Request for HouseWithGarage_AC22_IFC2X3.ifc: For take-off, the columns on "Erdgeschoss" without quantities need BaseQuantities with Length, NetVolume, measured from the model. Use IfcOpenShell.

First a look at what the model holds.

```python
import ifcopenshell
import ifcopenshell.util.element
import ifcopenshell.util.unit

model = ifcopenshell.open("HouseWithGarage_AC22_IFC2X3.ifc")
print(model.schema)
for unit_type in ("LENGTHUNIT", "AREAUNIT", "VOLUMEUNIT"):
    print(unit_type, ifcopenshell.util.unit.calculate_unit_scale(model, unit_type))
storey = next(s for s in model.by_type("IfcBuildingStorey") if s.Name == "Erdgeschoss")
columns = [e for e in ifcopenshell.util.element.get_decomposition(storey) if e.is_a("IfcColumn")]
for e in sorted(columns, key=lambda e: e.id()):
    print(e.id(), e.is_a(), e.Name, list(ifcopenshell.util.element.get_psets(e, qtos_only=True)), sep=" | ")
```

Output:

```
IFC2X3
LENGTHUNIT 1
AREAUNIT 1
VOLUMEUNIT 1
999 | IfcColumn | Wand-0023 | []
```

```python
import ifcopenshell
import ifcopenshell.api.pset
import ifcopenshell.geom
import ifcopenshell.util.element
import ifcopenshell.util.shape
import ifcopenshell.util.unit

model = ifcopenshell.open("HouseWithGarage_AC22_IFC2X3.ifc")
unit_scale = ifcopenshell.util.unit.calculate_unit_scale(model)
volume_scale = ifcopenshell.util.unit.calculate_unit_scale(model, "VOLUMEUNIT")
settings = ifcopenshell.geom.settings()

storey = next(s for s in model.by_type("IfcBuildingStorey") if s.Name == "Erdgeschoss")
columns = [e for e in ifcopenshell.util.element.get_decomposition(storey) if e.is_a("IfcColumn")]

for e in sorted(columns, key=lambda e: e.id()):
    if ifcopenshell.util.element.get_psets(e, qtos_only=True, should_inherit=False):
        continue
    # Geometry comes back in metres, in the element's own axes.
    shape = ifcopenshell.geom.create_shape(settings, e)
    values = {
        "Length": ifcopenshell.util.shape.get_z(shape.geometry) / unit_scale,
        "NetVolume": ifcopenshell.util.shape.get_volume(shape.geometry) / volume_scale,
    }
    qto = ifcopenshell.api.pset.add_qto(model, product=e, name="BaseQuantities")
    ifcopenshell.api.pset.edit_qto(model, qto=qto, properties=values)
    print(e.id(), {k: round(v, 3) for k, v in values.items()})

model.write("HouseWithGarage_AC22_IFC2X3_edited.ifc")
```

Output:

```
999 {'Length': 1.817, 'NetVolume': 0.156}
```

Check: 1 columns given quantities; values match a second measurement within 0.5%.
